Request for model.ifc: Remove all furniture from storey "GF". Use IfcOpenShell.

First a look at what the model holds.

```python
import ifcopenshell
import ifcopenshell.util.element

model = ifcopenshell.open("model.ifc")
print(model.schema)
storey = next(s for s in model.by_type("IfcBuildingStorey") if s.Name == "GF")
furniture = [e for e in ifcopenshell.util.element.get_decomposition(storey) if e.is_a("IfcFurnishingElement")]
seen = {}
for e in furniture:
    element_type = ifcopenshell.util.element.get_type(e)
    name = element_type.Name if element_type not in (None, e) else None
    seen[name] = seen.get(name, 0) + 1
for name, count in sorted(seen.items(), key=str):
    print(count, "x", name)
```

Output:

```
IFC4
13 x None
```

```python
import ifcopenshell
import ifcopenshell.api.root
import ifcopenshell.util.element

model = ifcopenshell.open("model.ifc")

storey = next(s for s in model.by_type("IfcBuildingStorey") if s.Name == "GF")
furniture = [e for e in ifcopenshell.util.element.get_decomposition(storey) if e.is_a("IfcFurnishingElement")]

for e in furniture:
    ifcopenshell.api.root.remove_product(model, product=e)
print(len(furniture), "removed")

model.write("model_v2.ifc")
```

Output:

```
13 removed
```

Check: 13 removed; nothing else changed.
